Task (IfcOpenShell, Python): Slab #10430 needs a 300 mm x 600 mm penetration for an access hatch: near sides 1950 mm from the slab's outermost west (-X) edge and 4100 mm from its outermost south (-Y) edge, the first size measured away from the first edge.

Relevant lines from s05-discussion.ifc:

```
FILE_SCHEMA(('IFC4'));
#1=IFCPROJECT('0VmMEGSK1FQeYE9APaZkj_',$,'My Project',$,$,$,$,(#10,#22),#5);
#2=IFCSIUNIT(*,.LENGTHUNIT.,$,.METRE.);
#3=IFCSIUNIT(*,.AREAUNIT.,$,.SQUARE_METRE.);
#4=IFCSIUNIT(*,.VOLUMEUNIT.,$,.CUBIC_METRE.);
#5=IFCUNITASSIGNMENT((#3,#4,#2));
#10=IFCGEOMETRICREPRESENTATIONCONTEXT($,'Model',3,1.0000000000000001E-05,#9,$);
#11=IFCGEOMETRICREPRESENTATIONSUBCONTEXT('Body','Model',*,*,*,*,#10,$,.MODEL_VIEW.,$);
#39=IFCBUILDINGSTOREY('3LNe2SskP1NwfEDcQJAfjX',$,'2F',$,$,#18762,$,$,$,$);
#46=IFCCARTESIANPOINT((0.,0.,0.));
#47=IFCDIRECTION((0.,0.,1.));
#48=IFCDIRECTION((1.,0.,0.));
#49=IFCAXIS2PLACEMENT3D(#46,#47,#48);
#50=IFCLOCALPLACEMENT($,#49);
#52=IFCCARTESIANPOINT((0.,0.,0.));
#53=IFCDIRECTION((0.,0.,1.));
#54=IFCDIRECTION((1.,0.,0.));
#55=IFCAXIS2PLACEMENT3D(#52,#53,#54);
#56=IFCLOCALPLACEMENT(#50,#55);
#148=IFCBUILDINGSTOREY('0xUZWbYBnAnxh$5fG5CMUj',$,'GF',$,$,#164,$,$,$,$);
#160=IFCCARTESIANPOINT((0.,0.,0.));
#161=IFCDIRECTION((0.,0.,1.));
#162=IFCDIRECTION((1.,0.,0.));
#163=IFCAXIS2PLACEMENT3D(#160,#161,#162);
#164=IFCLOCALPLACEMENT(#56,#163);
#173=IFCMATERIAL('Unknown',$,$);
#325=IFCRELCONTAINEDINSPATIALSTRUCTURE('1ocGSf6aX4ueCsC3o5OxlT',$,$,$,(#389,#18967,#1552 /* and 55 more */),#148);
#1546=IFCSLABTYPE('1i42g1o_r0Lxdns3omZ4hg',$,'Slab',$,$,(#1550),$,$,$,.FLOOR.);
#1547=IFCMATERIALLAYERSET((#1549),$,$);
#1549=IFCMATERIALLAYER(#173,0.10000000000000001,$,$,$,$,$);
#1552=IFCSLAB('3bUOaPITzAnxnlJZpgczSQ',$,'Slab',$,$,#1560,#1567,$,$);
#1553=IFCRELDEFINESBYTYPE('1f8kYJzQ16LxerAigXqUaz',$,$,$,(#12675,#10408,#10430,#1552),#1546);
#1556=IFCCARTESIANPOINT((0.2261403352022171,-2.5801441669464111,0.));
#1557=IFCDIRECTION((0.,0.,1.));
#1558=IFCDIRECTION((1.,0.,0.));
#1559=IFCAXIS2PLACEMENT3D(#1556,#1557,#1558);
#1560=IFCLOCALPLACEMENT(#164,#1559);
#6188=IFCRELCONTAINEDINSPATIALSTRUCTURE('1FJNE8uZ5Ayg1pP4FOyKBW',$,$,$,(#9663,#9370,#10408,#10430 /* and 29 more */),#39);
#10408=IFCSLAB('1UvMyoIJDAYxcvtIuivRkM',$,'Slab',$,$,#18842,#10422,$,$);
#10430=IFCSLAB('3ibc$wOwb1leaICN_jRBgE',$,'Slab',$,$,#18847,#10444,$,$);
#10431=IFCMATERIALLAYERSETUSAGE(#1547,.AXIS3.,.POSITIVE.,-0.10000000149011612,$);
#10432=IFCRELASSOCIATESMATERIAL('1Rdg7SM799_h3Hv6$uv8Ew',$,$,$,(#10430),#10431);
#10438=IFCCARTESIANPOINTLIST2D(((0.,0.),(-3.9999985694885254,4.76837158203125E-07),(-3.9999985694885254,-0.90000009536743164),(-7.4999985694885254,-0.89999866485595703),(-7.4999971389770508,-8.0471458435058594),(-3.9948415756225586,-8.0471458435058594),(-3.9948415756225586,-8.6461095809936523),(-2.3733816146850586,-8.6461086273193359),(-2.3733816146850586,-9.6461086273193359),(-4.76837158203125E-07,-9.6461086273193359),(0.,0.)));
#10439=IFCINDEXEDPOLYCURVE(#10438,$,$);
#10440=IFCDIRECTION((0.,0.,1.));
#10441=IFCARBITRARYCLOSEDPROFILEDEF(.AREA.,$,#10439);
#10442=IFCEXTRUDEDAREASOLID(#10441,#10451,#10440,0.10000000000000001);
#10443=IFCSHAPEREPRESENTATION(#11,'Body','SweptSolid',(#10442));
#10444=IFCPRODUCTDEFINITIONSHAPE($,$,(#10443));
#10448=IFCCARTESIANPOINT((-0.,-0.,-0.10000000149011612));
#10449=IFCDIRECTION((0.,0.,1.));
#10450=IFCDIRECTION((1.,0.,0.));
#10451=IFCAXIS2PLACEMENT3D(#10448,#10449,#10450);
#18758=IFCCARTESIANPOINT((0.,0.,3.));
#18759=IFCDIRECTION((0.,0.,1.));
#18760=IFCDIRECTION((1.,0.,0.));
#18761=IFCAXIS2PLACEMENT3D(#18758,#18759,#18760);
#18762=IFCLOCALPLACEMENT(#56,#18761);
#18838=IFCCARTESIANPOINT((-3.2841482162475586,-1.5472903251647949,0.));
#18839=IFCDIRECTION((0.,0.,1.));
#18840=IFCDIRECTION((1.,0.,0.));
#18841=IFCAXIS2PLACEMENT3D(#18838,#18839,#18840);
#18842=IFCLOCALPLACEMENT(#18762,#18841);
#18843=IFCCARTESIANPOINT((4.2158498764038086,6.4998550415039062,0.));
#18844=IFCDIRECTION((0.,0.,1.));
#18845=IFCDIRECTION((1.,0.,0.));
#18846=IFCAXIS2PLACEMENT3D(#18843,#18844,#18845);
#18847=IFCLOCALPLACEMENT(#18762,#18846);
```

```python
import numpy as np
import ifcopenshell
import ifcopenshell.api.feature
import ifcopenshell.api.geometry
import ifcopenshell.api.root
import ifcopenshell.geom
import ifcopenshell.util.placement
import ifcopenshell.util.representation
import ifcopenshell.util.shape
import ifcopenshell.util.unit

model = ifcopenshell.open("s05-discussion.ifc")
unit_scale = ifcopenshell.util.unit.calculate_unit_scale(model)
settings = ifcopenshell.geom.settings()


def volume(element):
    """Net volume in cubic metres, openings subtracted."""
    shape = ifcopenshell.geom.create_shape(settings, element)
    return ifcopenshell.util.shape.get_volume(shape.geometry)


slab = model.by_id(10430)
before = volume(slab)

# Extent in the slab's own axes, in metres. The edges named are its -X and -Y sides.
slab_shape = ifcopenshell.geom.create_shape(settings, slab)
vertices = ifcopenshell.util.shape.get_vertices(slab_shape.geometry)
x_min, y_min, bottom = vertices.min(axis=0)
top = vertices[:, 2].max()

opening = ifcopenshell.api.root.create_entity(model, ifc_class="IfcOpeningElement", name="Access hatch opening", predefined_type="OPENING")
context = ifcopenshell.util.representation.get_context(model, "Model", "Body", "MODEL_VIEW")
width, depth = 0.3, 0.6
outline = [(0.0, 0.0), (width, 0.0), (width, depth), (0.0, depth), (0.0, 0.0)]
# Overshoot both faces by 50 mm so the cut is clean.
shape = ifcopenshell.api.geometry.add_slab_representation(
    model, context=context, depth=top - bottom + 0.1, polyline=outline
)
ifcopenshell.api.geometry.assign_representation(model, product=opening, representation=shape)

matrix = ifcopenshell.util.placement.get_local_placement(slab.ObjectPlacement)
matrix[:, 3] = matrix @ np.append(np.array([x_min + 1.95, y_min + 4.1, bottom - 0.05]) / unit_scale, 1.0)
ifcopenshell.api.geometry.edit_object_placement(model, product=opening, matrix=matrix, is_si=False)
ifcopenshell.api.feature.add_feature(model, feature=opening, element=slab)

after = volume(slab)

print(f"slab volume {before:.3f} -> {after:.3f} m3")

model.write("s05-discussion-out.ifc")
```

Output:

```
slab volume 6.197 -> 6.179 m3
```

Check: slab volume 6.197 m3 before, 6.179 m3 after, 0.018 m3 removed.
